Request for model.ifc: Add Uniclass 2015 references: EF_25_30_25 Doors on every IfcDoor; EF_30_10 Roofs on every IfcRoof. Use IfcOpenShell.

First a look at what the model holds.

```python
import ifcopenshell

model = ifcopenshell.open("model.ifc")
print(model.schema)
print("classifications:", [c.Name for c in model.by_type("IfcClassification")])
for ifc_class in ("IfcDoor", "IfcRoof", "IfcStair", "IfcWall", "IfcWindow"):
    print(ifc_class, len(model.by_type(ifc_class)))
```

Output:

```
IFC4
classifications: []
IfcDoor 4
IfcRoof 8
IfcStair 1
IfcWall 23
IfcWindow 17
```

```python
import ifcopenshell
import ifcopenshell.api.classification

model = ifcopenshell.open("model.ifc")

system = ifcopenshell.api.classification.add_classification(model, classification="Uniclass 2015")

codes = {
    "IfcDoor": ("EF_25_30_25", "Doors"),
    "IfcRoof": ("EF_30_10", "Roofs"),
}
for ifc_class, (code, name) in codes.items():
    products = model.by_type(ifc_class)
    ifcopenshell.api.classification.add_reference(
        model, products=products, classification=system, identification=code, name=name
    )
    print(code, len(products))

model.write("model_edited.ifc")
```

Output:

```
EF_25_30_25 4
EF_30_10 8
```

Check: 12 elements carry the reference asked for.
